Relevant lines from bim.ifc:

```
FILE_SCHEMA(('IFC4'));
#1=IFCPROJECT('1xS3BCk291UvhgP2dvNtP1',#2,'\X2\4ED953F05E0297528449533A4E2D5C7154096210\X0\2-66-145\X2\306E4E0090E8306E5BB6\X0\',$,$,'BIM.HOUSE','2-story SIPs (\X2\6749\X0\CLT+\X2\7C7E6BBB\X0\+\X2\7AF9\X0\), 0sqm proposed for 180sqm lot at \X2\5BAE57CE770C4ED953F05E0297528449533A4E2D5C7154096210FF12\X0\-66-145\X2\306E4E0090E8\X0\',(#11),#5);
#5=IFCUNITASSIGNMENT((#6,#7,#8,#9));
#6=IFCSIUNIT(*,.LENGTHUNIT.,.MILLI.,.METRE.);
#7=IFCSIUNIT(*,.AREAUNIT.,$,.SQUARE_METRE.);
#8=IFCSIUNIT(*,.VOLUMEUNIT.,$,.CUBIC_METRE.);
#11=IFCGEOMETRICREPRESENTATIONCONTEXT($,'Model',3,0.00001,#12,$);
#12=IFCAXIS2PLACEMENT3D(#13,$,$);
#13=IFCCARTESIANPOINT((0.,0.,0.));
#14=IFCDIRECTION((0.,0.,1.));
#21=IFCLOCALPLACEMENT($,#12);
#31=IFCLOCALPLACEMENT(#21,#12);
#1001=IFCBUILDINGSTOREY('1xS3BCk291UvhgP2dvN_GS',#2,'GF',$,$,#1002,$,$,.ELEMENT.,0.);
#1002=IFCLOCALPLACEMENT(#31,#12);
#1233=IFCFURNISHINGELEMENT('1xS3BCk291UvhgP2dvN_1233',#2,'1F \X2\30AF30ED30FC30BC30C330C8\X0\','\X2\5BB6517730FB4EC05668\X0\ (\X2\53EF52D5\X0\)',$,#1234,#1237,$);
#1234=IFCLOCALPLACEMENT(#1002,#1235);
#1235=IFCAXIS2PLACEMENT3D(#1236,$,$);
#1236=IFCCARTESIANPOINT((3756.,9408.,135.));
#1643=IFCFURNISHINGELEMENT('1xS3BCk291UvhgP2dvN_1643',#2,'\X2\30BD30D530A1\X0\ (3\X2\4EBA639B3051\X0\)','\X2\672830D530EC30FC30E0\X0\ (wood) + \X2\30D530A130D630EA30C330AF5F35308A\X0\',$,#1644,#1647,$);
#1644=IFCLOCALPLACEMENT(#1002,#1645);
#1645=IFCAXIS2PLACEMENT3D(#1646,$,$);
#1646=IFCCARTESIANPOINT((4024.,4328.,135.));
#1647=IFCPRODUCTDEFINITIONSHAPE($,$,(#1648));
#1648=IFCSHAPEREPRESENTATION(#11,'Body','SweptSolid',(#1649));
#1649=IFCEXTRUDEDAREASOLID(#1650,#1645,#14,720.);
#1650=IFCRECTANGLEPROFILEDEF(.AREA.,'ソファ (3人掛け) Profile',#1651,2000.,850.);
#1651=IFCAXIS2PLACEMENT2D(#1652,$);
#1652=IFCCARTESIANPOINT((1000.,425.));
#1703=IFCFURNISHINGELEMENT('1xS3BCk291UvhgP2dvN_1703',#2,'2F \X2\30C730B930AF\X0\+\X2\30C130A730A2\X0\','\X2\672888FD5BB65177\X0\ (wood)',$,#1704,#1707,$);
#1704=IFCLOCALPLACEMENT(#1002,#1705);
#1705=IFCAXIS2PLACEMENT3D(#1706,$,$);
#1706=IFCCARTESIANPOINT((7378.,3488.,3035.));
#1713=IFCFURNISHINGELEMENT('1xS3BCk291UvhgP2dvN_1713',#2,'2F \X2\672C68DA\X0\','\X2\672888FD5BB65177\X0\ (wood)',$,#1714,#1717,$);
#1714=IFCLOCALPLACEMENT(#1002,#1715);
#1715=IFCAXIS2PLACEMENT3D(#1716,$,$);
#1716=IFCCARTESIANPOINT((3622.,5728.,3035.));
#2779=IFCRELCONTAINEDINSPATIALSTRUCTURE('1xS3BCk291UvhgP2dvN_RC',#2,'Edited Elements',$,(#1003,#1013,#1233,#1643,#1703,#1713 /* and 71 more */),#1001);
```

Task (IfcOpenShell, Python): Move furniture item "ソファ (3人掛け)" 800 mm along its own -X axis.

```python
import ifcopenshell
import ifcopenshell.api.geometry
import ifcopenshell.util.placement
import ifcopenshell.util.unit

model = ifcopenshell.open("bim.ifc")
unit_scale = ifcopenshell.util.unit.calculate_unit_scale(model)

item = model.by_guid("1xS3BCk291UvhgP2dvN_1643")
matrix = ifcopenshell.util.placement.get_local_placement(item.ObjectPlacement)
matrix[:3, 3] -= matrix[:3, 0] * 0.8 / unit_scale
ifcopenshell.api.geometry.edit_object_placement(model, product=item, matrix=matrix, is_si=False)

print(ifcopenshell.util.placement.get_local_placement(item.ObjectPlacement).round(3) + 0.0)

model.write("bim-out.ifc")
```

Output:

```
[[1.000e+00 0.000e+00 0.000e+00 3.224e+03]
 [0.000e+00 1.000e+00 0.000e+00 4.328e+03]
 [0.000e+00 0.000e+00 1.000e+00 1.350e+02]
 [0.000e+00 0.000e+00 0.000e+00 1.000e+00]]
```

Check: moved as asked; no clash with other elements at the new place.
